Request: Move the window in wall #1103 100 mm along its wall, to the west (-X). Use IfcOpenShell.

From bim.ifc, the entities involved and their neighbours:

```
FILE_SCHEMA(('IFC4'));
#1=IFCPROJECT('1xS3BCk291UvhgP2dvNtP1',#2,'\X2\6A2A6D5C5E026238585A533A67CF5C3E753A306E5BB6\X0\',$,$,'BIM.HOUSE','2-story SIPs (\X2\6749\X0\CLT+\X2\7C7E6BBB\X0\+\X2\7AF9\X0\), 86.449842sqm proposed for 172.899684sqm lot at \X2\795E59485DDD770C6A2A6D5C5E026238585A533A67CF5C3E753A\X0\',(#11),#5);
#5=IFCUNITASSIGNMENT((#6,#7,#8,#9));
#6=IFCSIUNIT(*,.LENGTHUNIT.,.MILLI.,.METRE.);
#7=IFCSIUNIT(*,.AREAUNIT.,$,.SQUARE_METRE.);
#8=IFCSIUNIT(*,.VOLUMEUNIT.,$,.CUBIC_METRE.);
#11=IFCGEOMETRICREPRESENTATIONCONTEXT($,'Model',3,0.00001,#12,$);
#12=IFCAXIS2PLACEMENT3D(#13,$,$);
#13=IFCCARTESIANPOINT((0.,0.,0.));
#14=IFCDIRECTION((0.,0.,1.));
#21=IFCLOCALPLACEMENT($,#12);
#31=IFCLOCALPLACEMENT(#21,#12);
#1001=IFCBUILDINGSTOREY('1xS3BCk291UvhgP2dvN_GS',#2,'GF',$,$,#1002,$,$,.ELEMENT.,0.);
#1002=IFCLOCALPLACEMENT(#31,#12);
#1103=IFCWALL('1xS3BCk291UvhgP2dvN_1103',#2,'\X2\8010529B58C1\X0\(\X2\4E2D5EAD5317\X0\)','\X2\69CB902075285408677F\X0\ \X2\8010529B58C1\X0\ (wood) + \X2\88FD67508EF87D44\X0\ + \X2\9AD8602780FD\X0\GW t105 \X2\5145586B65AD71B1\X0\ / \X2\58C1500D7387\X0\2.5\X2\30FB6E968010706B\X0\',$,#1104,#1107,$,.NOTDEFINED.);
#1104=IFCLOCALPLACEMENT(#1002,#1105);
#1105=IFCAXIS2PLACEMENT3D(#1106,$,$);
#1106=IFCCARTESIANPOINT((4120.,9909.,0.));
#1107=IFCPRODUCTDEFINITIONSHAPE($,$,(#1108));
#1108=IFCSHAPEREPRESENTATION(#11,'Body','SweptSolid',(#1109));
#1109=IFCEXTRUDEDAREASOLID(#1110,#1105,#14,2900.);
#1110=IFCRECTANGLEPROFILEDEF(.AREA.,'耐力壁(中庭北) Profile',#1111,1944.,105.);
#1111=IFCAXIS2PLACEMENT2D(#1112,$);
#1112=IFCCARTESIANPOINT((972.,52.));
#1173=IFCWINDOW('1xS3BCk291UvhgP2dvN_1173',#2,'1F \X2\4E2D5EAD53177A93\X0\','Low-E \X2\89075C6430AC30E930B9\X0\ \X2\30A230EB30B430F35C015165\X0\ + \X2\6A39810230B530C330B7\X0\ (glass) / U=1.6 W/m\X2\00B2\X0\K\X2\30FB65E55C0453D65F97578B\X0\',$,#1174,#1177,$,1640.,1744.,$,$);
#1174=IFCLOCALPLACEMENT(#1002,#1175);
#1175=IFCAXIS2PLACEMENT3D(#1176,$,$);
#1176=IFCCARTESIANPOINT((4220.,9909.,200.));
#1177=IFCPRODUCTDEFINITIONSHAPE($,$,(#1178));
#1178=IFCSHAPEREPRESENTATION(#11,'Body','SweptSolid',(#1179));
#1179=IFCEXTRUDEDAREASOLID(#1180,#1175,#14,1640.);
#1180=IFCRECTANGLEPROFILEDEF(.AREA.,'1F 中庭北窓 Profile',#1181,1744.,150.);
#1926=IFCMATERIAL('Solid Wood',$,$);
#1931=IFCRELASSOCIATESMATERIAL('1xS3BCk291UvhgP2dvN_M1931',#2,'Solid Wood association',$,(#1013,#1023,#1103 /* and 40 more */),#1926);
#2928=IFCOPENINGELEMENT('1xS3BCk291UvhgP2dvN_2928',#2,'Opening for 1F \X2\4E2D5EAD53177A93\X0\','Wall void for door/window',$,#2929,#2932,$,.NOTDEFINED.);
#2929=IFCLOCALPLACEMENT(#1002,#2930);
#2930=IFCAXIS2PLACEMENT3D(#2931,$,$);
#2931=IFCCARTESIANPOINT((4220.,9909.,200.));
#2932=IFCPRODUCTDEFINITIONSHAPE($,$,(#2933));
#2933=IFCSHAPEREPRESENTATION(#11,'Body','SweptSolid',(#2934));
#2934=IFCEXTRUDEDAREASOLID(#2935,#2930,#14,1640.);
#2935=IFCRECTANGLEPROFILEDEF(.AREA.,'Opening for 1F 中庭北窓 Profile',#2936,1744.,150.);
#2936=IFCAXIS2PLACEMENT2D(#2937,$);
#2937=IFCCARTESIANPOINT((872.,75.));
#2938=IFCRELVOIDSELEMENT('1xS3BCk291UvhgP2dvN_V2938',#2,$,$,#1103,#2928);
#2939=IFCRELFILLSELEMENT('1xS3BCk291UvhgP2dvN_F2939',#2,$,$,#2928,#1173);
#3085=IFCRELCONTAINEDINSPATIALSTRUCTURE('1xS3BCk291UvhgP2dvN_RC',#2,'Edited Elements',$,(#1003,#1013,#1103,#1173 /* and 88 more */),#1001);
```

```python
import ifcopenshell
import ifcopenshell.api.geometry
import ifcopenshell.util.placement
import ifcopenshell.util.unit

model = ifcopenshell.open("bim.ifc")
unit_scale = ifcopenshell.util.unit.calculate_unit_scale(model)

window = model.by_guid("1xS3BCk291UvhgP2dvN_1173")
opening = window.FillsVoids[0].RelatingOpeningElement
wall = opening.VoidsElements[0].RelatingBuildingElement

wall_matrix = ifcopenshell.util.placement.get_local_placement(wall.ObjectPlacement)
shift = wall_matrix[:3, 0] * -0.1 / unit_scale
before = ifcopenshell.util.placement.get_local_placement(window.ObjectPlacement)[:3, 3].copy()

# The window is not placed relative to its opening, so move both.
for product in (opening, window):
    matrix = ifcopenshell.util.placement.get_local_placement(product.ObjectPlacement)
    matrix[:3, 3] += shift
    ifcopenshell.api.geometry.edit_object_placement(model, product=product, matrix=matrix, is_si=False)

after = ifcopenshell.util.placement.get_local_placement(window.ObjectPlacement)[:3, 3]
print("window moved by", (after - before).round(3) + 0.0)

model.write("bim-out.ifc")
```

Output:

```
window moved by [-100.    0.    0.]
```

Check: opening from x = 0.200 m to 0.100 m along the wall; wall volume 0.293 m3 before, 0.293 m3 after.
